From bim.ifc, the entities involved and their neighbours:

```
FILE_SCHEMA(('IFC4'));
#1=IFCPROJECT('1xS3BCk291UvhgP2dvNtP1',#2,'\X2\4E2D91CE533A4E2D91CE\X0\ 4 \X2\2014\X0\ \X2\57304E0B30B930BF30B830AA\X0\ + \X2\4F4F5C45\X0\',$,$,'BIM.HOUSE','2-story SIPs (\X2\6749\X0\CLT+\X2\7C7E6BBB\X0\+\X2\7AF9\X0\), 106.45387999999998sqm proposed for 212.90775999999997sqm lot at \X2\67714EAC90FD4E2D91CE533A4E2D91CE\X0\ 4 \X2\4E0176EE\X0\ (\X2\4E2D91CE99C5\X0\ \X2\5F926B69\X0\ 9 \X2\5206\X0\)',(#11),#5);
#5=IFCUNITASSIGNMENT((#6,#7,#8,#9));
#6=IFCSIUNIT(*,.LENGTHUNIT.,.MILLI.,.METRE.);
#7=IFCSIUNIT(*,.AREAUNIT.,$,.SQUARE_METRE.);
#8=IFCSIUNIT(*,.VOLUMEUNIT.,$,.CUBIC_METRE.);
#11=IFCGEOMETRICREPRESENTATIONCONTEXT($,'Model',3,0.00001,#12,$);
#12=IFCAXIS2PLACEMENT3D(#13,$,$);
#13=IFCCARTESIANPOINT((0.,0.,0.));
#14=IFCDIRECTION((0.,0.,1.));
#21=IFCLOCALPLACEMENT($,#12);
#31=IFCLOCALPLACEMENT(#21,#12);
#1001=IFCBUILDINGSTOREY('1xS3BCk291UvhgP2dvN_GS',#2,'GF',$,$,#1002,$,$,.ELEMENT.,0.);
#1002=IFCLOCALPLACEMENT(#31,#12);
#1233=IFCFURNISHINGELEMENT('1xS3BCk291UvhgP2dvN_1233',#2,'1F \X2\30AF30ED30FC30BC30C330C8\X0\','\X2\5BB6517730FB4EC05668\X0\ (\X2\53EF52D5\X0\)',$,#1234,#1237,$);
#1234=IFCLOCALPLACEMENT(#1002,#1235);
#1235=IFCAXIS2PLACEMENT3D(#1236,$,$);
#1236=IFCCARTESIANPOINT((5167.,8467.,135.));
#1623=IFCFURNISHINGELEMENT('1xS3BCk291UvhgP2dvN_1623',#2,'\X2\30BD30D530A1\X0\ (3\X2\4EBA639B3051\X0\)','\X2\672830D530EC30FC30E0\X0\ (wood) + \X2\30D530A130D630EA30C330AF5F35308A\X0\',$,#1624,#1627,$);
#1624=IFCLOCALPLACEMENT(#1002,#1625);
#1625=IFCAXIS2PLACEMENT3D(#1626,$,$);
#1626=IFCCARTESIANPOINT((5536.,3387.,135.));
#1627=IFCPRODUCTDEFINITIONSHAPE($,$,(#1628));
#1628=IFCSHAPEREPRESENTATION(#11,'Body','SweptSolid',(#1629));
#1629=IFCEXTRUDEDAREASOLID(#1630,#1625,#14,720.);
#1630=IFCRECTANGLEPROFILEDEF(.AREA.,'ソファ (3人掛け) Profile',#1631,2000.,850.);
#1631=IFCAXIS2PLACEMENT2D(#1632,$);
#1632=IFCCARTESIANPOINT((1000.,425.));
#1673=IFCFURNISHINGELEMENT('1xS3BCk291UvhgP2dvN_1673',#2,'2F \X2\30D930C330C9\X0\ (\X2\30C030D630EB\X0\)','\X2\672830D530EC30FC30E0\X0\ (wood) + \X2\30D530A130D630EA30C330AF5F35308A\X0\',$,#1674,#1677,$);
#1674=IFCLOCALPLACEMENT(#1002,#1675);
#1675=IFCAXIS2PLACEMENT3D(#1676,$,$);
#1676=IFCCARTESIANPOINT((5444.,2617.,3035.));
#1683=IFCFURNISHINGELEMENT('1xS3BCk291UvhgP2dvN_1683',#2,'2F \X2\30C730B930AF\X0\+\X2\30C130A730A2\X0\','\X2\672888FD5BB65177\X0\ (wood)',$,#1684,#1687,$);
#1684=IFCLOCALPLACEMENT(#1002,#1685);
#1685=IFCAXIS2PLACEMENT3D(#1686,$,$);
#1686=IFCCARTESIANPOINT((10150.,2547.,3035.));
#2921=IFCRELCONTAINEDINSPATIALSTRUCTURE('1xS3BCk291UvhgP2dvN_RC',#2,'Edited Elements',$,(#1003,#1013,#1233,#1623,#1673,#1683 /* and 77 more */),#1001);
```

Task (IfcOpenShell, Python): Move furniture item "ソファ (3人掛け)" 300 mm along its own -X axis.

```python
import ifcopenshell
import ifcopenshell.api.geometry
import ifcopenshell.util.placement

model = ifcopenshell.open("bim.ifc")

item = model.by_id(1623)
matrix = ifcopenshell.util.placement.get_local_placement(item.ObjectPlacement)
matrix[:3, 3] -= matrix[:3, 0] * 300.0
ifcopenshell.api.geometry.edit_object_placement(model, product=item, matrix=matrix, is_si=False)

print(ifcopenshell.util.placement.get_local_placement(item.ObjectPlacement).round(3) + 0.0)

model.write("bim_rev.ifc")
```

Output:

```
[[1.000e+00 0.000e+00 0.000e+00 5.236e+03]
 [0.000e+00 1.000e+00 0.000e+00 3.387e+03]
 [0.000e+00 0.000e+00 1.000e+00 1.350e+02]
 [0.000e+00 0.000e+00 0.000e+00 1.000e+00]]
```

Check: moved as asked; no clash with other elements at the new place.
